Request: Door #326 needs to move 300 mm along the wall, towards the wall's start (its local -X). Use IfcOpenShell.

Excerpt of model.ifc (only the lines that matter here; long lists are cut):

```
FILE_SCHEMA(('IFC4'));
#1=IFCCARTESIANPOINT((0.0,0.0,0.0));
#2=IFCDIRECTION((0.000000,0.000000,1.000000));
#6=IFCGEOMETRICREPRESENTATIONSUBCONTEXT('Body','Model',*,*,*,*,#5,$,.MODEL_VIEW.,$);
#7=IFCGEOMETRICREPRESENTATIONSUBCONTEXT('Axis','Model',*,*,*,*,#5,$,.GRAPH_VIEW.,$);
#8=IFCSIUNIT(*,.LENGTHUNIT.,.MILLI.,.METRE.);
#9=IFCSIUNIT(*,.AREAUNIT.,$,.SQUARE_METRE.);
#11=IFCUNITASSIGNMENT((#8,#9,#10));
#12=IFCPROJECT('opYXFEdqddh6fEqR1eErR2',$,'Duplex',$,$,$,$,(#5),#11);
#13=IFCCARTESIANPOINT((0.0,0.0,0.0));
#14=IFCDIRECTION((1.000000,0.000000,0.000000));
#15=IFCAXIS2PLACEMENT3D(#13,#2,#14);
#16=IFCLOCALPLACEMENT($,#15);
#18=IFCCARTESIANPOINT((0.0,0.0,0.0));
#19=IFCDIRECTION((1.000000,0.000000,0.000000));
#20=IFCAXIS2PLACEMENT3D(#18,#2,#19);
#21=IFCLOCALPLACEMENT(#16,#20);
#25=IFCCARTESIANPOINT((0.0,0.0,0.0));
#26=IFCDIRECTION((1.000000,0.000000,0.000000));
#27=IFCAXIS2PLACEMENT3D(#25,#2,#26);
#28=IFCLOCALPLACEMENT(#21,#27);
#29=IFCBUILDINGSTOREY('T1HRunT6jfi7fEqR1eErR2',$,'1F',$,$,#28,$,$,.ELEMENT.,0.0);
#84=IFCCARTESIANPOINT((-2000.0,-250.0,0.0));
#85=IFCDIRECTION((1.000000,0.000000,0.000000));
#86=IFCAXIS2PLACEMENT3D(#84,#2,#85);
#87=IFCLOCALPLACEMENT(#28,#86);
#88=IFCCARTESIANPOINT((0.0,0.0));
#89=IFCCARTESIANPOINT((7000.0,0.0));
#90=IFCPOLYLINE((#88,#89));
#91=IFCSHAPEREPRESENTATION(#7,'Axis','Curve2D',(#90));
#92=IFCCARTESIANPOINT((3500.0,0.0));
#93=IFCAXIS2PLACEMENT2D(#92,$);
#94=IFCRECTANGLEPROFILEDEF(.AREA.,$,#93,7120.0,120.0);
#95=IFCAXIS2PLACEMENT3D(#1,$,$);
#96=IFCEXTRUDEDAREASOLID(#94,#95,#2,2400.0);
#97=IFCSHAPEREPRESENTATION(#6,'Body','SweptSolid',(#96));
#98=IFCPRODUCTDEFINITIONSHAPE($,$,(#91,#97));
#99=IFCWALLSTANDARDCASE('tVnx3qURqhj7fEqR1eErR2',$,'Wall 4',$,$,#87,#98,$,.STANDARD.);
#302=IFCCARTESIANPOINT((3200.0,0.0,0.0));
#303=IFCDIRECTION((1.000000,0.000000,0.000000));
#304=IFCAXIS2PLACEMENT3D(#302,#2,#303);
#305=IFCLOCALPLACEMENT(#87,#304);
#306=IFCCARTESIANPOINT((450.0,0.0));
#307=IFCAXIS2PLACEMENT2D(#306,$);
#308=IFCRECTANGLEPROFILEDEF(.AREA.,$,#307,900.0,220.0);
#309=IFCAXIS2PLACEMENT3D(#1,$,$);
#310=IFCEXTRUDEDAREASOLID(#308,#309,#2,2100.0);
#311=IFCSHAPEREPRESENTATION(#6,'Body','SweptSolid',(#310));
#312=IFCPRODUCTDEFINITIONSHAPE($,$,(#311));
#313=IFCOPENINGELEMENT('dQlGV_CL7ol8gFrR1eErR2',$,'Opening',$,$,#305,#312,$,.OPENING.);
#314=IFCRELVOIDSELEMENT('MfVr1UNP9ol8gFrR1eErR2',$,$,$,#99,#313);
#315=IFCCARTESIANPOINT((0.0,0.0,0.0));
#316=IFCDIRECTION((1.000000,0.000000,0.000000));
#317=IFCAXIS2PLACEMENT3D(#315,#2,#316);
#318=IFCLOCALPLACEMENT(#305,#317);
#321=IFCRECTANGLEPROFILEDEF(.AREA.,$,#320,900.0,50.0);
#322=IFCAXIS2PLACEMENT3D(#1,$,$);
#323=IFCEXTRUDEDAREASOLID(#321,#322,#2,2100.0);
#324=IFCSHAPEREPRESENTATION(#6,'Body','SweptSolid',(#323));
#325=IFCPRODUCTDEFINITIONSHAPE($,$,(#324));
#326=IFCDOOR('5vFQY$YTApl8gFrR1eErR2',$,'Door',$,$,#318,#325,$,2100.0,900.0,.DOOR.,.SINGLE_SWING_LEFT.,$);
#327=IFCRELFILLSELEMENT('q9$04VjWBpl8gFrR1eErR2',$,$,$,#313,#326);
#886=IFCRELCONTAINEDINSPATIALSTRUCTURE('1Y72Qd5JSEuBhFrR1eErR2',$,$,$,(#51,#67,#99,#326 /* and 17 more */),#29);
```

```python
import ifcopenshell
import ifcopenshell.api.geometry
import ifcopenshell.util.placement
import ifcopenshell.util.unit

model = ifcopenshell.open("model.ifc")
unit_scale = ifcopenshell.util.unit.calculate_unit_scale(model)

door = model.by_guid("5vFQY$YTApl8gFrR1eErR2")
opening = door.FillsVoids[0].RelatingOpeningElement
wall = opening.VoidsElements[0].RelatingBuildingElement

wall_matrix = ifcopenshell.util.placement.get_local_placement(wall.ObjectPlacement)
shift = wall_matrix[:3, 0] * -0.3 / unit_scale
before = ifcopenshell.util.placement.get_local_placement(door.ObjectPlacement)[:3, 3].copy()

# The door is placed relative to its opening, so it follows when the opening moves.
matrix = ifcopenshell.util.placement.get_local_placement(opening.ObjectPlacement)
matrix[:3, 3] += shift
ifcopenshell.api.geometry.edit_object_placement(
    model, product=opening, matrix=matrix, is_si=False, should_transform_children=True
)

after = ifcopenshell.util.placement.get_local_placement(door.ObjectPlacement)[:3, 3]
print("door moved by", (after - before).round(3) + 0.0)

model.write("model_edited.ifc")
```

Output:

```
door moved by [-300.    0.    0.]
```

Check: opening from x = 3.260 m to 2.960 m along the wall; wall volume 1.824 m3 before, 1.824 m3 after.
